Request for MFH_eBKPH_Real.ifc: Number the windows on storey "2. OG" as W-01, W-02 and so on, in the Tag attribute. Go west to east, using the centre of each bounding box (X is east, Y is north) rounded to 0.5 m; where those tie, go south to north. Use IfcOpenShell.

First a look at what the model holds.

```python
import ifcopenshell
import ifcopenshell.util.element
import ifcopenshell.util.placement

model = ifcopenshell.open("MFH_eBKPH_Real.ifc")
print(model.schema)
storey = next(s for s in model.by_type("IfcBuildingStorey") if s.Name == "2. OG")
windows = [e for e in ifcopenshell.util.element.get_decomposition(storey) if e.is_a("IfcWindow")]
for e in sorted(windows, key=lambda e: e.id()):
    origin = ifcopenshell.util.placement.get_local_placement(e.ObjectPlacement)[:3, 3]
    print(e.id(), e.Tag, e.Name, origin.round(2) + 0.0, sep=" | ")
```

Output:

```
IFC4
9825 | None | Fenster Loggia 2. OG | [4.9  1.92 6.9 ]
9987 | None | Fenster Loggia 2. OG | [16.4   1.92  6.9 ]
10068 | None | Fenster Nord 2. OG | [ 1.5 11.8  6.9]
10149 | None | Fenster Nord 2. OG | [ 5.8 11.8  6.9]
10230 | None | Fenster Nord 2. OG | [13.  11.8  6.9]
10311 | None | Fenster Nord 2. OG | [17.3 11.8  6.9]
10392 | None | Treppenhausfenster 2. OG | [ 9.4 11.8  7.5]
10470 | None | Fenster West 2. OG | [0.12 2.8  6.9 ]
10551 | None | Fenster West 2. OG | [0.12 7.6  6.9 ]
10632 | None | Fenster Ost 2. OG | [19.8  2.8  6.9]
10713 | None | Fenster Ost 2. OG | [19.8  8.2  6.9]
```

```python
import ifcopenshell
import ifcopenshell.geom
import ifcopenshell.util.element
import ifcopenshell.util.shape

model = ifcopenshell.open("MFH_eBKPH_Real.ifc")
settings = ifcopenshell.geom.settings()
settings.set("use-world-coords", True)


def centre(element):
    shape = ifcopenshell.geom.create_shape(settings, element)
    return ifcopenshell.util.shape.get_bbox_centroid(shape.geometry)


storey = next(s for s in model.by_type("IfcBuildingStorey") if s.Name == "2. OG")
windows = [e for e in ifcopenshell.util.element.get_decomposition(storey) if e.is_a("IfcWindow")]

# Insertion points can sit at a corner or the storey origin, so sort by the geometry (in metres).
centres = {e: centre(e) for e in windows}
windows.sort(key=lambda e: (round(centres[e][0] / 0.5), centres[e][1]))

for i, e in enumerate(windows, start=1):
    number = f"W-{i:02d}"
    e.Tag = number
    print(e.id(), number)

model.write("MFH_eBKPH_Real-out.ifc")
```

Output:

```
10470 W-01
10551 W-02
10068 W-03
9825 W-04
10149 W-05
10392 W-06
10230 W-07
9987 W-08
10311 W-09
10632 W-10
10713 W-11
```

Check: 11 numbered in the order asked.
